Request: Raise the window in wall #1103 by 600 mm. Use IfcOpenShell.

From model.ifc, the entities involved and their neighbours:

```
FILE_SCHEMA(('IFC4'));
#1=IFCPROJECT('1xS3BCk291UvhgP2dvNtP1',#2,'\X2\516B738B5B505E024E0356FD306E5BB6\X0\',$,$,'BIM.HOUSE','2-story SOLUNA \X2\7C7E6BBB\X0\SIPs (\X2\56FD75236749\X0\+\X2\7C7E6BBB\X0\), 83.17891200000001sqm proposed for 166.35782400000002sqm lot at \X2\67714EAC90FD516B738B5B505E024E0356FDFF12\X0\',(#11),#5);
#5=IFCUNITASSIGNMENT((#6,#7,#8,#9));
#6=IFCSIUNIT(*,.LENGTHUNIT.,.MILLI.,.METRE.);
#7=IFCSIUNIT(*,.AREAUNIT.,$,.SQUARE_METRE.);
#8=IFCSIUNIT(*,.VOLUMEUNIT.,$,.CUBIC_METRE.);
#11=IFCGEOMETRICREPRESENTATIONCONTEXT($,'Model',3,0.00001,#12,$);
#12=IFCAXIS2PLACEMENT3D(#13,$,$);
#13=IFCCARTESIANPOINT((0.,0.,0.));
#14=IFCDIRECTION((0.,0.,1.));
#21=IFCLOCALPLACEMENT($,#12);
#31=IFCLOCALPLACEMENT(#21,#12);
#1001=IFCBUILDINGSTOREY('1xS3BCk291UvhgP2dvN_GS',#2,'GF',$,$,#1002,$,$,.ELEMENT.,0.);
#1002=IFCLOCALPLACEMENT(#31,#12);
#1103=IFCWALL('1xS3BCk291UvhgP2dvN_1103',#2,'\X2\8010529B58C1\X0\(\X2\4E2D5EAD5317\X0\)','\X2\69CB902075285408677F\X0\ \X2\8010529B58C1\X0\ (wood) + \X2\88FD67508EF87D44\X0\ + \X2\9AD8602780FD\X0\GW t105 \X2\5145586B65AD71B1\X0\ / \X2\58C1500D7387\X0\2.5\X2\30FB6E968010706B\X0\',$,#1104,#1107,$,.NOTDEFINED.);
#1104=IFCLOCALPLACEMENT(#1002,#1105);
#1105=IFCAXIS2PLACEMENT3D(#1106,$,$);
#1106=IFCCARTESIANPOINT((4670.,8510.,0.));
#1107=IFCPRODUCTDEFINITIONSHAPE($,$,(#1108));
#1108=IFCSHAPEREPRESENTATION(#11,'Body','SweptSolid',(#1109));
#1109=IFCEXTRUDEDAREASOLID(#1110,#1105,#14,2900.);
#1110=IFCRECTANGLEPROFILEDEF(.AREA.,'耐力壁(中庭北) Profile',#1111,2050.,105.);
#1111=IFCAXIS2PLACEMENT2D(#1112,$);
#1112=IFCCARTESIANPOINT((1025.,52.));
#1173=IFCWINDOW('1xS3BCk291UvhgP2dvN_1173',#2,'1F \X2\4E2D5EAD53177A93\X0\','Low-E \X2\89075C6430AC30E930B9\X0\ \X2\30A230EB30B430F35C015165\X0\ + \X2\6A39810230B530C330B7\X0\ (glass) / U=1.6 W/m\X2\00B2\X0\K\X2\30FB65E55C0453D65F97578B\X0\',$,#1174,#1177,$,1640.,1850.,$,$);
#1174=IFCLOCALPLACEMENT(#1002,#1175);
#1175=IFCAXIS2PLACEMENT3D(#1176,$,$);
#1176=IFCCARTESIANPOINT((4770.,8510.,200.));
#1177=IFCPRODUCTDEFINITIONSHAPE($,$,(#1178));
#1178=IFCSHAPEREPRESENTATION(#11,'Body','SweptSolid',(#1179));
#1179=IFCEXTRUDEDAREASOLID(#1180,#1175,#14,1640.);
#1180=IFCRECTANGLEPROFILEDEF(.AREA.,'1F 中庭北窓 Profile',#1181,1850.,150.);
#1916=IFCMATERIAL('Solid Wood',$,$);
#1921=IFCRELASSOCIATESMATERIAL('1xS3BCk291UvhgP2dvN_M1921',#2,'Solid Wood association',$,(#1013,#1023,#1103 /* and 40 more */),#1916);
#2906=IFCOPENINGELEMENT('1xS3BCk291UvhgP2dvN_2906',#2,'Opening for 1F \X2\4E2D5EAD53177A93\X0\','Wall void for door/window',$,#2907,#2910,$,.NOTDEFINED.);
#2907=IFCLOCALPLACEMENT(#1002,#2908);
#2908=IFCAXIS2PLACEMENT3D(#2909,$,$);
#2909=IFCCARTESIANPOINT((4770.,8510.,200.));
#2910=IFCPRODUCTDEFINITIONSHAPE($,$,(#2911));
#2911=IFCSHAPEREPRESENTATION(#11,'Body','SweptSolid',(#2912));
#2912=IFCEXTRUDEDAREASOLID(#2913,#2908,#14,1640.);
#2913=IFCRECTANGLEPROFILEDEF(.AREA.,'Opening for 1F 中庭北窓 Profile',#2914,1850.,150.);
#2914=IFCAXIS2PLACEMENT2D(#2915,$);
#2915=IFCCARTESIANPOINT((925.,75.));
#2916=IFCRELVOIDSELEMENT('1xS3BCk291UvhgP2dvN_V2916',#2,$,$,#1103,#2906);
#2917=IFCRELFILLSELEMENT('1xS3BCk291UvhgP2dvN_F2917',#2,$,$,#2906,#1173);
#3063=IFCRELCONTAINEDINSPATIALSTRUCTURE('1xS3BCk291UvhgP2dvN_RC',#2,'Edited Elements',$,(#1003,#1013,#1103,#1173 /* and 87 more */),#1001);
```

```python
import numpy as np
import ifcopenshell
import ifcopenshell.api.geometry
import ifcopenshell.util.placement
import ifcopenshell.util.unit

model = ifcopenshell.open("model.ifc")
unit_scale = ifcopenshell.util.unit.calculate_unit_scale(model)

window = model.by_guid("1xS3BCk291UvhgP2dvN_1173")
opening = window.FillsVoids[0].RelatingOpeningElement
dz = 0.6 / unit_scale

shift = np.array([0.0, 0.0, dz])
# The window is not placed relative to its opening, so move both.
for product in (opening, window):
    matrix = ifcopenshell.util.placement.get_local_placement(product.ObjectPlacement)
    matrix[:3, 3] += shift
    ifcopenshell.api.geometry.edit_object_placement(model, product=product, matrix=matrix, is_si=False)

print(f"moved by {dz * unit_scale:+.3f} m")

model.write("model_edited.ifc")
```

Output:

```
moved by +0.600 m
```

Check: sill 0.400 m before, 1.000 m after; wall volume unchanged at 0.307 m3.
